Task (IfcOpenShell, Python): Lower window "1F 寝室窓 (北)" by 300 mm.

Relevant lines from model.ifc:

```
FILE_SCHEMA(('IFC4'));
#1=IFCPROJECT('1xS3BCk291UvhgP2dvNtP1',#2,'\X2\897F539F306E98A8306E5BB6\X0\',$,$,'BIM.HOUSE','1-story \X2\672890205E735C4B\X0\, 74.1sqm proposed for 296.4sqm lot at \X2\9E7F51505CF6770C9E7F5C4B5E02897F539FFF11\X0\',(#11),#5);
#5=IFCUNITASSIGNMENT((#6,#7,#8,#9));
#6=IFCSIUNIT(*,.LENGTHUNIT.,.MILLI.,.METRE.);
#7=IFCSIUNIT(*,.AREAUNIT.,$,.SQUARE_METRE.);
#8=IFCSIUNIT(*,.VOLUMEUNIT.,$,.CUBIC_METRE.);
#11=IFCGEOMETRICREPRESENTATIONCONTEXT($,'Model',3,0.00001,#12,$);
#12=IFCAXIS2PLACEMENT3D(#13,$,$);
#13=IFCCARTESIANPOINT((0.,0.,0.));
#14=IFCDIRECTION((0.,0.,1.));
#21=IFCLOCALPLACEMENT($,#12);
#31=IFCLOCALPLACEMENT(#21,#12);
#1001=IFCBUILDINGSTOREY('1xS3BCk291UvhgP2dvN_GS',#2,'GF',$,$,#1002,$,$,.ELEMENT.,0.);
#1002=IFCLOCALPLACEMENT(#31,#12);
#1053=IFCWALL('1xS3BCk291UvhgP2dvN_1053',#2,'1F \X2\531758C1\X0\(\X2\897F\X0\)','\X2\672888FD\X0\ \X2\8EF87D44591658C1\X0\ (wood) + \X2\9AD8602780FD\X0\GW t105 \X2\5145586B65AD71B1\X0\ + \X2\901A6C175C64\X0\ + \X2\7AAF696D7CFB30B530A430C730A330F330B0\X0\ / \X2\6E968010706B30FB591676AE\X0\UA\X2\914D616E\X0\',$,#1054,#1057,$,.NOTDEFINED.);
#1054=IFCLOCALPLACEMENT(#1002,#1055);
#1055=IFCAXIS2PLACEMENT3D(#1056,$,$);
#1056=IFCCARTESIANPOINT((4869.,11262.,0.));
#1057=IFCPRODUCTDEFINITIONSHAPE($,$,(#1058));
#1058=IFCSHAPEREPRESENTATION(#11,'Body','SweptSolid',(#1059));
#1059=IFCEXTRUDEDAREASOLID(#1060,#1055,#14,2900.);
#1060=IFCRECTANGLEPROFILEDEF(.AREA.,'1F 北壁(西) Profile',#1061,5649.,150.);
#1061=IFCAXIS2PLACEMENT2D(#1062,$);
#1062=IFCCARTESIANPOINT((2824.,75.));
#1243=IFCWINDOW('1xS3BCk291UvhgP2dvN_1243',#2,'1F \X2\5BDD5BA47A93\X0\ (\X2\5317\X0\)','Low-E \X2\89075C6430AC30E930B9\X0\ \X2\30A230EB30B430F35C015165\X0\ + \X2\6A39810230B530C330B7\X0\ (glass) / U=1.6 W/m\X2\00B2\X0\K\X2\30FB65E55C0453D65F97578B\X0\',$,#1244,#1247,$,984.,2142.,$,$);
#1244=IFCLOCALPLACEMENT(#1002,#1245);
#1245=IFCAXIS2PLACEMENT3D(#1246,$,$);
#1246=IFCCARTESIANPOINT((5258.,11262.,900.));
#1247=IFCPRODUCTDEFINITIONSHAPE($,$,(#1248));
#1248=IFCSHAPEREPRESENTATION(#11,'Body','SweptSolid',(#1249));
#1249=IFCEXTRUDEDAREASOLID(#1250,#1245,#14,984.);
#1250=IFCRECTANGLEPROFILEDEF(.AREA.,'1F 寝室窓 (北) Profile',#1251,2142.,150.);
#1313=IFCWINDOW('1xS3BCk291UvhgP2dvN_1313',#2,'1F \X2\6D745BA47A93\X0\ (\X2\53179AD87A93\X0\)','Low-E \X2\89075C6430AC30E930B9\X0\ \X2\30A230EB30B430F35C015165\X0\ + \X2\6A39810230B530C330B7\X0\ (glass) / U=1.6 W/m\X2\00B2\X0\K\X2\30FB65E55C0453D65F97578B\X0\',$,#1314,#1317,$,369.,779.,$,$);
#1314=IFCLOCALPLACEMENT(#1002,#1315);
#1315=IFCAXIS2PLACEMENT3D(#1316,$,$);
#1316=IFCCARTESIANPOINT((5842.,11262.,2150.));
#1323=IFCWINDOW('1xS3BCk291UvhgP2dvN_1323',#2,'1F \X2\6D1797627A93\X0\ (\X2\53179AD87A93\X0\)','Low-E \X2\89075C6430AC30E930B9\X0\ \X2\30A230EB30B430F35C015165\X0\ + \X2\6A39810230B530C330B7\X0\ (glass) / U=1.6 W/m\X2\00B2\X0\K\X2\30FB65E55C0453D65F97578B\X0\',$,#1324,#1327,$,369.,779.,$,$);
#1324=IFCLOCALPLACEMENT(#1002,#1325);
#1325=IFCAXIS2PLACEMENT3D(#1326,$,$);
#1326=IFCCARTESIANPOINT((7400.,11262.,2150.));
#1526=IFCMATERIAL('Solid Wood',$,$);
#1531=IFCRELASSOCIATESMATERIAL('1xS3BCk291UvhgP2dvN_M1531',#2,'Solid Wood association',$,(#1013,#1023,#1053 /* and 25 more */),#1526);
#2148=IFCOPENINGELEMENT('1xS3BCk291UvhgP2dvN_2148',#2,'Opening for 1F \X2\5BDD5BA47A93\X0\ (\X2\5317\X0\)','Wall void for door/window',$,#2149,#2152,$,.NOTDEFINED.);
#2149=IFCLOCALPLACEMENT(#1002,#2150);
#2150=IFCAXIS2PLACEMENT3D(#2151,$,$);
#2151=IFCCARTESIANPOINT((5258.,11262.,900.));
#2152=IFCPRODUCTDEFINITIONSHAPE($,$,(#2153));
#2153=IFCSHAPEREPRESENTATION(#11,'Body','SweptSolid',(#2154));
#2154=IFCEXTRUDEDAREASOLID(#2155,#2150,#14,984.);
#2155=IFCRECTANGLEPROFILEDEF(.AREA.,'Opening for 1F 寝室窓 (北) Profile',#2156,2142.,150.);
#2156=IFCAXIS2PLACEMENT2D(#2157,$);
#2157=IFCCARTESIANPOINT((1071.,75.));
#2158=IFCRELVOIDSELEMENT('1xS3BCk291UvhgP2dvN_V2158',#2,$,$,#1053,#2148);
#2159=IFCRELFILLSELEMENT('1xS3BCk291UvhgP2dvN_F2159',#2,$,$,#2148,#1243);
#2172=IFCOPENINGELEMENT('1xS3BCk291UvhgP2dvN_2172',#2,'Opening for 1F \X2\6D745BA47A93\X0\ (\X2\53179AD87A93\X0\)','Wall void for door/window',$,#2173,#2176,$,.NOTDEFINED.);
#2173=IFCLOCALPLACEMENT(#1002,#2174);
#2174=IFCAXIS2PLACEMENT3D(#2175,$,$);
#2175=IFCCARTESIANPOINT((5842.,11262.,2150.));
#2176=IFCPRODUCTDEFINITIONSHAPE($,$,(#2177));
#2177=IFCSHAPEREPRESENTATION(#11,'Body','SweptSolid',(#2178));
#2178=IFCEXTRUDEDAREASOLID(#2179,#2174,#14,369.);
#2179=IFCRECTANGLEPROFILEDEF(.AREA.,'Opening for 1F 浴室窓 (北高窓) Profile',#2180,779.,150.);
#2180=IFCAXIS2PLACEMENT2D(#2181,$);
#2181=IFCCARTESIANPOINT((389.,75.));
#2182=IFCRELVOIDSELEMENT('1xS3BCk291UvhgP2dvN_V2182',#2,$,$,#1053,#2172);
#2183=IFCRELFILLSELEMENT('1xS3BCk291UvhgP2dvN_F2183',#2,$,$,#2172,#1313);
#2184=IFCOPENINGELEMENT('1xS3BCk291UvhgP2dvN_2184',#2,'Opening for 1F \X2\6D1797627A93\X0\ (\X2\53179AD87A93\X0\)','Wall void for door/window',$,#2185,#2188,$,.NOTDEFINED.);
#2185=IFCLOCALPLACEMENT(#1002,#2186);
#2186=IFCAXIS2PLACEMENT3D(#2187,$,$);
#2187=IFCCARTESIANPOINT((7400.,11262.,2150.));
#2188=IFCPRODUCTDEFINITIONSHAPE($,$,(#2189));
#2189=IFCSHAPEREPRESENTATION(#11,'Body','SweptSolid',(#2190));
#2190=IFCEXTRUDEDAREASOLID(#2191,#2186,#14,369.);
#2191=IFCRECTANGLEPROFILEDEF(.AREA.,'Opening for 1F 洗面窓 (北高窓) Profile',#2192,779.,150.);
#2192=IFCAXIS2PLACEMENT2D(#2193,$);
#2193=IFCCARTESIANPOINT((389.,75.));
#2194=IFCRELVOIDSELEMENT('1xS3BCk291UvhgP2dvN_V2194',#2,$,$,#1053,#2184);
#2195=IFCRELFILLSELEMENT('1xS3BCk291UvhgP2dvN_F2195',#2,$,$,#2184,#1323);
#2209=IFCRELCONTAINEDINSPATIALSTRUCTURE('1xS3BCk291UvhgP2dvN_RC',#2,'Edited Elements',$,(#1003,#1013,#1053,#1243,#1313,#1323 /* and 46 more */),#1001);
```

```python
import numpy as np
import ifcopenshell
import ifcopenshell.api.geometry
import ifcopenshell.util.placement
import ifcopenshell.util.unit

model = ifcopenshell.open("model.ifc")
unit_scale = ifcopenshell.util.unit.calculate_unit_scale(model)

window = model.by_id(1243)
opening = window.FillsVoids[0].RelatingOpeningElement
dz = -300.0

shift = np.array([0.0, 0.0, dz])
# The window is not placed relative to its opening, so move both.
for product in (opening, window):
    matrix = ifcopenshell.util.placement.get_local_placement(product.ObjectPlacement)
    matrix[:3, 3] += shift
    ifcopenshell.api.geometry.edit_object_placement(model, product=product, matrix=matrix, is_si=False)

print(f"moved by {dz * unit_scale:+.3f} m")

model.write("model_v2.ifc")
```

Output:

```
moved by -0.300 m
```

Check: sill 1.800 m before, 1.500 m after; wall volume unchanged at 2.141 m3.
